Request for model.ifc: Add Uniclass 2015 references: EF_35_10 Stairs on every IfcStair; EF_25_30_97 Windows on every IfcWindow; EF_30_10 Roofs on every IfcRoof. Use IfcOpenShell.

First a look at what the model holds.

```python
import ifcopenshell

model = ifcopenshell.open("model.ifc")
print(model.schema)
print("classifications:", [c.Name for c in model.by_type("IfcClassification")])
for ifc_class in ("IfcDoor", "IfcRoof", "IfcStair", "IfcWall", "IfcWindow"):
    print(ifc_class, len(model.by_type(ifc_class)))
```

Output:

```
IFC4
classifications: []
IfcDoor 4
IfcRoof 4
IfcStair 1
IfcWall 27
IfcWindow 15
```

```python
import ifcopenshell
import ifcopenshell.api.classification

model = ifcopenshell.open("model.ifc")

system = ifcopenshell.api.classification.add_classification(model, classification="Uniclass 2015")

codes = {
    "IfcStair": ("EF_35_10", "Stairs"),
    "IfcWindow": ("EF_25_30_97", "Windows"),
    "IfcRoof": ("EF_30_10", "Roofs"),
}
for ifc_class, (code, name) in codes.items():
    products = model.by_type(ifc_class)
    ifcopenshell.api.classification.add_reference(
        model, products=products, classification=system, identification=code, name=name
    )
    print(code, len(products))

model.write("model_rev.ifc")
```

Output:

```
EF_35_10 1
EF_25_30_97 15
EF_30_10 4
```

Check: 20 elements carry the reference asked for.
